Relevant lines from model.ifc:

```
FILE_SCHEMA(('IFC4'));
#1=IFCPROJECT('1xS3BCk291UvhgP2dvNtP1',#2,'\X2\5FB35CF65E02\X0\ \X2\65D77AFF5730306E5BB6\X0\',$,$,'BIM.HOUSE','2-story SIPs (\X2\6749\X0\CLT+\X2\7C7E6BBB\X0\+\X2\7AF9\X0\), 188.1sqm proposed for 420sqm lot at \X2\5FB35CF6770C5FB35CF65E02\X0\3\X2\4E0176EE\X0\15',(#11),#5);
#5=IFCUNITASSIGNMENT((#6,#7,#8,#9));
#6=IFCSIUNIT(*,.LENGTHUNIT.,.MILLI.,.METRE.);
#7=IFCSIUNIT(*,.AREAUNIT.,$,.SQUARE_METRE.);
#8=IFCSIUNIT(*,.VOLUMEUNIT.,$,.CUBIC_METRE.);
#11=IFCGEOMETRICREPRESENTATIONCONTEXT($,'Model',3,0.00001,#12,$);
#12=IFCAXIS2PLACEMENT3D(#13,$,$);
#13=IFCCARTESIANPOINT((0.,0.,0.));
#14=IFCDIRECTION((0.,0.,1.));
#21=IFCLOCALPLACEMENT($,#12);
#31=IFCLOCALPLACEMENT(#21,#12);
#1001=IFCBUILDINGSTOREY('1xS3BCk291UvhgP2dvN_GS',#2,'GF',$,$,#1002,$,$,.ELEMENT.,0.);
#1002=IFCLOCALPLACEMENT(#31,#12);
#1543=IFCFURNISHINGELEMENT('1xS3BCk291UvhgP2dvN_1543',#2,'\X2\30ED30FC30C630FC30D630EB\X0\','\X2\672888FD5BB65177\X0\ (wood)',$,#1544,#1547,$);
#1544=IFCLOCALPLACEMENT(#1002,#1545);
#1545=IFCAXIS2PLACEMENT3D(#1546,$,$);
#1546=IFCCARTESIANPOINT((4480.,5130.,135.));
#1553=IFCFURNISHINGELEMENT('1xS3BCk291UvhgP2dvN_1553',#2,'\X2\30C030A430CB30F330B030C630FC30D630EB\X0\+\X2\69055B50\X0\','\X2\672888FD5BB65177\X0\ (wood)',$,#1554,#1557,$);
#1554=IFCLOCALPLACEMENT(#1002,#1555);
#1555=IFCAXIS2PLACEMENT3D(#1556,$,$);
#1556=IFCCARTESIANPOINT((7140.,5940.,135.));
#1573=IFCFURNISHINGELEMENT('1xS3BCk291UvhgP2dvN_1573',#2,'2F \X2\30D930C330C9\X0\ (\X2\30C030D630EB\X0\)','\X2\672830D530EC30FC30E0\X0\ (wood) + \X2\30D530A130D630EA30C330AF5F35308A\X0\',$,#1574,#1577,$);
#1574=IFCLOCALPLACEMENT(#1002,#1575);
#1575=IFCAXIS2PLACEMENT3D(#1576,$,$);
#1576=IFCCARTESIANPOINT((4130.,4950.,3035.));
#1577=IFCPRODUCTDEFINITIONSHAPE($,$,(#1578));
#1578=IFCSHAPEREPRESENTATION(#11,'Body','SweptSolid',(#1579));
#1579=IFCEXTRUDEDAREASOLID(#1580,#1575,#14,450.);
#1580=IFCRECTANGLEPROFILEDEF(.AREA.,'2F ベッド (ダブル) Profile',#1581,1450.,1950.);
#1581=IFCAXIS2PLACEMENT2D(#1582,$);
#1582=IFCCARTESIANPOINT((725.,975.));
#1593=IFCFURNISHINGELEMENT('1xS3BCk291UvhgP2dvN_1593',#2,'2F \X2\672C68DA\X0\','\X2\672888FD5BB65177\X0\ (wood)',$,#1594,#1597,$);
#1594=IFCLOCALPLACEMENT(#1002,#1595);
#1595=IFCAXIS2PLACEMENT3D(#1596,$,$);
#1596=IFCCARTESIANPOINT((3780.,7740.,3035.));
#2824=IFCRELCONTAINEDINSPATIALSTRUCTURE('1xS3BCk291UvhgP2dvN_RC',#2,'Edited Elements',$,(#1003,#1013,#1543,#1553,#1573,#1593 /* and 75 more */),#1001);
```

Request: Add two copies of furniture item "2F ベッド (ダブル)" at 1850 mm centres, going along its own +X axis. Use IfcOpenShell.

```python
import ifcopenshell
import ifcopenshell.api.geometry
import ifcopenshell.api.root
import ifcopenshell.util.element
import ifcopenshell.util.placement

model = ifcopenshell.open("model.ifc")


def reuse_history(source, copy):
    """copy_class also copies each property set's owner history, people and application; keep the originals."""
    for rel in copy.IsDefinedBy:
        if rel.is_a("IfcRelDefinesByProperties") and (history := rel.RelatingPropertyDefinition.OwnerHistory):
            rel.RelatingPropertyDefinition.OwnerHistory = source.OwnerHistory
            ifcopenshell.util.element.remove_deep2(model, history)


source = model.by_guid("1xS3BCk291UvhgP2dvN_1573")
base = ifcopenshell.util.placement.get_local_placement(source.ObjectPlacement)
step = base[:3, 0] * 1850.0

for i in range(1, 3):
    copy = ifcopenshell.api.root.copy_class(model, product=source)
    copy.Representation = ifcopenshell.util.element.copy_deep(
        model, source.Representation, exclude=["IfcGeometricRepresentationContext", "IfcRepresentationMap"]
    )
    reuse_history(source, copy)
    matrix = base.copy()
    matrix[:3, 3] += i * step
    print("added at", matrix[:3, 3].round(3) + 0.0)
    ifcopenshell.api.geometry.edit_object_placement(model, product=copy, matrix=matrix, is_si=False)

model.write("model_edited.ifc")
```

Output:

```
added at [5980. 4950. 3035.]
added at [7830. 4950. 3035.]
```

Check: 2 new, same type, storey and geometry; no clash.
